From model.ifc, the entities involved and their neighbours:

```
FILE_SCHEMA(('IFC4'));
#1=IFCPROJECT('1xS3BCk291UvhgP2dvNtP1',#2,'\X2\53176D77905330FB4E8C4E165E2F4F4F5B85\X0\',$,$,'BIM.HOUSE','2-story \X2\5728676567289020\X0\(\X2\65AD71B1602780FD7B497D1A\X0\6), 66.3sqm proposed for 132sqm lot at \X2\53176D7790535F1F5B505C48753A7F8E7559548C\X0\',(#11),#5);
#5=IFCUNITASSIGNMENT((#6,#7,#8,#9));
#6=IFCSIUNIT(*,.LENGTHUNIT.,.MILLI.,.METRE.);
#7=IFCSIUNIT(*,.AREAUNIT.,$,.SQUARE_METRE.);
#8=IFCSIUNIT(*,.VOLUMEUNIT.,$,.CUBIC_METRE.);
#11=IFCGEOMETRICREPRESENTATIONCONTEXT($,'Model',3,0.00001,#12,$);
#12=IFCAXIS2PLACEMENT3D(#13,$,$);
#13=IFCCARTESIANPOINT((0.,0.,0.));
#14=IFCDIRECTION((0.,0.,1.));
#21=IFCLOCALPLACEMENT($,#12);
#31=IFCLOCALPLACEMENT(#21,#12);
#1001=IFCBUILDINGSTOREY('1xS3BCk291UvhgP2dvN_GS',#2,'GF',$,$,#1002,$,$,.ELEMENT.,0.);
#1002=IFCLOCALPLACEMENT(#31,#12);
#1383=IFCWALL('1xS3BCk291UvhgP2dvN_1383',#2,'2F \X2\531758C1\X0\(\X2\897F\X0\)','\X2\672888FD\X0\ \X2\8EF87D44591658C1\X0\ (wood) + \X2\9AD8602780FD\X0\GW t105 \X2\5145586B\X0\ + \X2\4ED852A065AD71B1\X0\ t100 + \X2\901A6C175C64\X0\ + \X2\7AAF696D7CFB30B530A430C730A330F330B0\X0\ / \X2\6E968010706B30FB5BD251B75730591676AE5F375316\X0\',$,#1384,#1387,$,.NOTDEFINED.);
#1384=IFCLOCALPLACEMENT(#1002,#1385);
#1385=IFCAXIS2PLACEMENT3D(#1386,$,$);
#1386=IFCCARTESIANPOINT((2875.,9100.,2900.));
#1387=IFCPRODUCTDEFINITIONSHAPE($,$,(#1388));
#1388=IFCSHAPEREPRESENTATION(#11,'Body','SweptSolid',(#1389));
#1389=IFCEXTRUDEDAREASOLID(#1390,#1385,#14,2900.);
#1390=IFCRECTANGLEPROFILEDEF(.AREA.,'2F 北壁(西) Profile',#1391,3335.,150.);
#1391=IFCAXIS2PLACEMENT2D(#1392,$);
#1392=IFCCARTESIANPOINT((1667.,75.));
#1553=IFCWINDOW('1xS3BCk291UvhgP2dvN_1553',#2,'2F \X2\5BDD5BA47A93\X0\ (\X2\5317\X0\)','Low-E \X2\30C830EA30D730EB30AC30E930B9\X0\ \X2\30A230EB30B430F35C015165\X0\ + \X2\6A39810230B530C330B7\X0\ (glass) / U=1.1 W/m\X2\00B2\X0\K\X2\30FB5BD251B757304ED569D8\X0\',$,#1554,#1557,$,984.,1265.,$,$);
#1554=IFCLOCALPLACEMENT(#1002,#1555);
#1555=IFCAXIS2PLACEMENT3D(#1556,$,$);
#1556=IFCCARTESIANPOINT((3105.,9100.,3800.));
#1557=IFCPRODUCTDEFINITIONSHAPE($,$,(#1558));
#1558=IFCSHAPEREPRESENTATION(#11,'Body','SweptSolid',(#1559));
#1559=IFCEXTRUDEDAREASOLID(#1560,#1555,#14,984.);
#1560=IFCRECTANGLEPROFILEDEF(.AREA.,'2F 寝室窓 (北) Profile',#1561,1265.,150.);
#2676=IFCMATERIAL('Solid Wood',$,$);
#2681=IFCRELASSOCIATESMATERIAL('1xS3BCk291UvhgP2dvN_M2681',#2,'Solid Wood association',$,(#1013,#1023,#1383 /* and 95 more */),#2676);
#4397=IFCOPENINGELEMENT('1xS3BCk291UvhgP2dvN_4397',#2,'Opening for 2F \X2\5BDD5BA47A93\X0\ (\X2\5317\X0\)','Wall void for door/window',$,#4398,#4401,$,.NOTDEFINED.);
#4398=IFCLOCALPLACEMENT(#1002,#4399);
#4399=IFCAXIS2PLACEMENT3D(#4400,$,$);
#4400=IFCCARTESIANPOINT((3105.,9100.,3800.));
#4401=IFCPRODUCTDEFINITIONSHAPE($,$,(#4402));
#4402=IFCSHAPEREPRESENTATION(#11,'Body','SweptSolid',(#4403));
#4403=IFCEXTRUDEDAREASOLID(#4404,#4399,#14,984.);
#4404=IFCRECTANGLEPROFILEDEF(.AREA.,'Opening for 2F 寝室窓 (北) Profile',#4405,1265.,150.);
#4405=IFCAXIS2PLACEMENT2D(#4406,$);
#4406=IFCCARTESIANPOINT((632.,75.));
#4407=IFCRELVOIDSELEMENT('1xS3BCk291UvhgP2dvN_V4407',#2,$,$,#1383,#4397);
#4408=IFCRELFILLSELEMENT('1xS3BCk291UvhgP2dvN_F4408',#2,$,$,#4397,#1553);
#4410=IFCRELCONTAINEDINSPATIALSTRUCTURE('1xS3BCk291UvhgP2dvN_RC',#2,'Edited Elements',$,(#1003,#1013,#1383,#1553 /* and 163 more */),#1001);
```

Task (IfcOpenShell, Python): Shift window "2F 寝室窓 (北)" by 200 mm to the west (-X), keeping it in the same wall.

```python
import ifcopenshell
import ifcopenshell.api.geometry
import ifcopenshell.util.placement

model = ifcopenshell.open("model.ifc")

window = model.by_guid("1xS3BCk291UvhgP2dvN_1553")
opening = window.FillsVoids[0].RelatingOpeningElement
wall = opening.VoidsElements[0].RelatingBuildingElement

wall_matrix = ifcopenshell.util.placement.get_local_placement(wall.ObjectPlacement)
shift = wall_matrix[:3, 0] * -200.0
before = ifcopenshell.util.placement.get_local_placement(window.ObjectPlacement)[:3, 3].copy()

# The window is not placed relative to its opening, so move both.
for product in (opening, window):
    matrix = ifcopenshell.util.placement.get_local_placement(product.ObjectPlacement)
    matrix[:3, 3] += shift
    ifcopenshell.api.geometry.edit_object_placement(model, product=product, matrix=matrix, is_si=False)

after = ifcopenshell.util.placement.get_local_placement(window.ObjectPlacement)[:3, 3]
print("window moved by", (after - before).round(3) + 0.0)

model.write("model_edited.ifc")
```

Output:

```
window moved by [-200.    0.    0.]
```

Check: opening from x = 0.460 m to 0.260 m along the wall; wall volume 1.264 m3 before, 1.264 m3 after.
